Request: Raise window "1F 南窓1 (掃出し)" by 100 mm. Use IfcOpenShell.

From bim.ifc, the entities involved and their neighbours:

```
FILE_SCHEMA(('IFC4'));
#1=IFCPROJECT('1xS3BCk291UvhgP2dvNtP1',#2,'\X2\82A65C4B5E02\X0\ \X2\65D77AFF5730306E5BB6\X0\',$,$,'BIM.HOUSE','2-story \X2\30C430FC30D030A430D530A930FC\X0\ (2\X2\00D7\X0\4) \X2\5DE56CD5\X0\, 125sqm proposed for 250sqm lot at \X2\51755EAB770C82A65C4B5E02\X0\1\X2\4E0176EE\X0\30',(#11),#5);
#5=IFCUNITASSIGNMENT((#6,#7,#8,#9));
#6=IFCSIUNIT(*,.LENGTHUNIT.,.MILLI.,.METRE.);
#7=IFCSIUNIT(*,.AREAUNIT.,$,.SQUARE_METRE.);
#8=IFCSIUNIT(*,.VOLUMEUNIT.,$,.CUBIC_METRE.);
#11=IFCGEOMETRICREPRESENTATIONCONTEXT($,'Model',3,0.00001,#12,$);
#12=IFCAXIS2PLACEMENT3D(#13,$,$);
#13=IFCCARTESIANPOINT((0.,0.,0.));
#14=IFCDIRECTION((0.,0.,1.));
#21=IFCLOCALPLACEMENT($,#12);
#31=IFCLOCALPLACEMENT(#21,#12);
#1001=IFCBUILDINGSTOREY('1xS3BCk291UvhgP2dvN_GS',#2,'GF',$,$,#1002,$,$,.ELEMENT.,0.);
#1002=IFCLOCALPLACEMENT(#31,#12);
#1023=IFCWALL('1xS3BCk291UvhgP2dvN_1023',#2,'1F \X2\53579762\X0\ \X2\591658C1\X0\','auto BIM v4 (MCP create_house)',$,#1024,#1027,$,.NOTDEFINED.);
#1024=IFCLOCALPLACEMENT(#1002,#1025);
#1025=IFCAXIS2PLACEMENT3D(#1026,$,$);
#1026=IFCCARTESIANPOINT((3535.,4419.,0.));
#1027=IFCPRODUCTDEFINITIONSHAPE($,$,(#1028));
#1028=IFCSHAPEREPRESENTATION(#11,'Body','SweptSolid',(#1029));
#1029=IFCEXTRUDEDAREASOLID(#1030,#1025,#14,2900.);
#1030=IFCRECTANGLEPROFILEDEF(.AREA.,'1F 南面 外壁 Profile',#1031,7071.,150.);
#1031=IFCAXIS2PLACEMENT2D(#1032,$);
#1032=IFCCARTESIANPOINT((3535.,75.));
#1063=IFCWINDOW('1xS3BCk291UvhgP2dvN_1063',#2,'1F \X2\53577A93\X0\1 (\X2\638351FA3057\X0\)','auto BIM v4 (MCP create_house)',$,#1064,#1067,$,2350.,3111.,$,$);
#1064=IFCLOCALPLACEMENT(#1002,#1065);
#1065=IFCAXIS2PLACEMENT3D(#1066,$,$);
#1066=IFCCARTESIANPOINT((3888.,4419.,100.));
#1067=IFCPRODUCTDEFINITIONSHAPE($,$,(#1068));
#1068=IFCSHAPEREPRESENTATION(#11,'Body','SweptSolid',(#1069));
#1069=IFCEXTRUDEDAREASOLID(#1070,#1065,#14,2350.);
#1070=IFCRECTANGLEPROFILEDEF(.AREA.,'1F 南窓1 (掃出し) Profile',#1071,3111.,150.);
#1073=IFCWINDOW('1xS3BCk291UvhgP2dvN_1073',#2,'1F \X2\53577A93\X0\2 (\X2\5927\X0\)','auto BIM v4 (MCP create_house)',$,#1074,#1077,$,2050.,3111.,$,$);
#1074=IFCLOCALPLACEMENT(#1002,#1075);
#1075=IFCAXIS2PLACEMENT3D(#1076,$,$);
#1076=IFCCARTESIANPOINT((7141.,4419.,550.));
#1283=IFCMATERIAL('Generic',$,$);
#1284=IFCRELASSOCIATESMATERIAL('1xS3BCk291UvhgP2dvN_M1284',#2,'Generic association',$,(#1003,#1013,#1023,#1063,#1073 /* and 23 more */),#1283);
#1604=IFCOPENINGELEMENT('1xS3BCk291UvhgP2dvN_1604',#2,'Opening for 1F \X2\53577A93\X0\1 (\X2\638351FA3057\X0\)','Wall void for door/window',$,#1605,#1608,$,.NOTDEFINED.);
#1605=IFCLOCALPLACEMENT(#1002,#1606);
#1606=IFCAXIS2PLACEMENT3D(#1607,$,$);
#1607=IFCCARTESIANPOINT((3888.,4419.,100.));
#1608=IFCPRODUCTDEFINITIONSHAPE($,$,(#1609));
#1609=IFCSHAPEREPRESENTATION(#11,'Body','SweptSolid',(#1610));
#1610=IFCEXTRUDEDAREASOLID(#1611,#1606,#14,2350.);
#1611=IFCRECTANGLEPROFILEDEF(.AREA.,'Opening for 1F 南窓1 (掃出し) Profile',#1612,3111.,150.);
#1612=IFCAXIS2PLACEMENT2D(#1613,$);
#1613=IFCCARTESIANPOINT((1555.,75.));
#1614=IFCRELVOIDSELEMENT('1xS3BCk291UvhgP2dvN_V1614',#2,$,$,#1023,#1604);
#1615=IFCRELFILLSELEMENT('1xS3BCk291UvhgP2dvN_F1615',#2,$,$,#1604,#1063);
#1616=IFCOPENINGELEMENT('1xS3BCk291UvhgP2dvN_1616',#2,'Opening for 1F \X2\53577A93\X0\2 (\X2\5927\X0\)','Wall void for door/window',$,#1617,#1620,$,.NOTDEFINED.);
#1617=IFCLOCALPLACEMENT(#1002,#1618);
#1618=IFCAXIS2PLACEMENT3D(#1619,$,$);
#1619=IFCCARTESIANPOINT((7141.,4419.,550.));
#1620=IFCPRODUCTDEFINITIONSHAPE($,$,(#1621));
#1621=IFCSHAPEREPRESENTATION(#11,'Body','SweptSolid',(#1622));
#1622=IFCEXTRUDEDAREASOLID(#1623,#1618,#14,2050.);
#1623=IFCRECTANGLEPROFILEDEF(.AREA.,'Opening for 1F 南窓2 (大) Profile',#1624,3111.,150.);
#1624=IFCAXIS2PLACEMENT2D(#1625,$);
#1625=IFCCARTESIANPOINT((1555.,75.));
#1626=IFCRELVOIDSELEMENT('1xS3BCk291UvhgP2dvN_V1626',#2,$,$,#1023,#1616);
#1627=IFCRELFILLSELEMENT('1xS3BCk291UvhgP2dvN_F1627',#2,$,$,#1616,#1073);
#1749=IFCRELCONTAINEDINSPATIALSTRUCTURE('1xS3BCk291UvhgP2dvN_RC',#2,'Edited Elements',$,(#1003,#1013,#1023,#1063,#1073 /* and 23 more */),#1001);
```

```python
import numpy as np
import ifcopenshell
import ifcopenshell.api.geometry
import ifcopenshell.util.placement
import ifcopenshell.util.unit

model = ifcopenshell.open("bim.ifc")
unit_scale = ifcopenshell.util.unit.calculate_unit_scale(model)

window = model.by_guid("1xS3BCk291UvhgP2dvN_1063")
opening = window.FillsVoids[0].RelatingOpeningElement
dz = 0.1 / unit_scale

shift = np.array([0.0, 0.0, dz])
# The window is not placed relative to its opening, so move both.
for product in (opening, window):
    matrix = ifcopenshell.util.placement.get_local_placement(product.ObjectPlacement)
    matrix[:3, 3] += shift
    ifcopenshell.api.geometry.edit_object_placement(model, product=product, matrix=matrix, is_si=False)

print(f"moved by {dz * unit_scale:+.3f} m")

model.write("bim_v2.ifc")
```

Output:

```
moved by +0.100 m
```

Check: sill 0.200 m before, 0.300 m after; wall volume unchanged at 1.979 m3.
